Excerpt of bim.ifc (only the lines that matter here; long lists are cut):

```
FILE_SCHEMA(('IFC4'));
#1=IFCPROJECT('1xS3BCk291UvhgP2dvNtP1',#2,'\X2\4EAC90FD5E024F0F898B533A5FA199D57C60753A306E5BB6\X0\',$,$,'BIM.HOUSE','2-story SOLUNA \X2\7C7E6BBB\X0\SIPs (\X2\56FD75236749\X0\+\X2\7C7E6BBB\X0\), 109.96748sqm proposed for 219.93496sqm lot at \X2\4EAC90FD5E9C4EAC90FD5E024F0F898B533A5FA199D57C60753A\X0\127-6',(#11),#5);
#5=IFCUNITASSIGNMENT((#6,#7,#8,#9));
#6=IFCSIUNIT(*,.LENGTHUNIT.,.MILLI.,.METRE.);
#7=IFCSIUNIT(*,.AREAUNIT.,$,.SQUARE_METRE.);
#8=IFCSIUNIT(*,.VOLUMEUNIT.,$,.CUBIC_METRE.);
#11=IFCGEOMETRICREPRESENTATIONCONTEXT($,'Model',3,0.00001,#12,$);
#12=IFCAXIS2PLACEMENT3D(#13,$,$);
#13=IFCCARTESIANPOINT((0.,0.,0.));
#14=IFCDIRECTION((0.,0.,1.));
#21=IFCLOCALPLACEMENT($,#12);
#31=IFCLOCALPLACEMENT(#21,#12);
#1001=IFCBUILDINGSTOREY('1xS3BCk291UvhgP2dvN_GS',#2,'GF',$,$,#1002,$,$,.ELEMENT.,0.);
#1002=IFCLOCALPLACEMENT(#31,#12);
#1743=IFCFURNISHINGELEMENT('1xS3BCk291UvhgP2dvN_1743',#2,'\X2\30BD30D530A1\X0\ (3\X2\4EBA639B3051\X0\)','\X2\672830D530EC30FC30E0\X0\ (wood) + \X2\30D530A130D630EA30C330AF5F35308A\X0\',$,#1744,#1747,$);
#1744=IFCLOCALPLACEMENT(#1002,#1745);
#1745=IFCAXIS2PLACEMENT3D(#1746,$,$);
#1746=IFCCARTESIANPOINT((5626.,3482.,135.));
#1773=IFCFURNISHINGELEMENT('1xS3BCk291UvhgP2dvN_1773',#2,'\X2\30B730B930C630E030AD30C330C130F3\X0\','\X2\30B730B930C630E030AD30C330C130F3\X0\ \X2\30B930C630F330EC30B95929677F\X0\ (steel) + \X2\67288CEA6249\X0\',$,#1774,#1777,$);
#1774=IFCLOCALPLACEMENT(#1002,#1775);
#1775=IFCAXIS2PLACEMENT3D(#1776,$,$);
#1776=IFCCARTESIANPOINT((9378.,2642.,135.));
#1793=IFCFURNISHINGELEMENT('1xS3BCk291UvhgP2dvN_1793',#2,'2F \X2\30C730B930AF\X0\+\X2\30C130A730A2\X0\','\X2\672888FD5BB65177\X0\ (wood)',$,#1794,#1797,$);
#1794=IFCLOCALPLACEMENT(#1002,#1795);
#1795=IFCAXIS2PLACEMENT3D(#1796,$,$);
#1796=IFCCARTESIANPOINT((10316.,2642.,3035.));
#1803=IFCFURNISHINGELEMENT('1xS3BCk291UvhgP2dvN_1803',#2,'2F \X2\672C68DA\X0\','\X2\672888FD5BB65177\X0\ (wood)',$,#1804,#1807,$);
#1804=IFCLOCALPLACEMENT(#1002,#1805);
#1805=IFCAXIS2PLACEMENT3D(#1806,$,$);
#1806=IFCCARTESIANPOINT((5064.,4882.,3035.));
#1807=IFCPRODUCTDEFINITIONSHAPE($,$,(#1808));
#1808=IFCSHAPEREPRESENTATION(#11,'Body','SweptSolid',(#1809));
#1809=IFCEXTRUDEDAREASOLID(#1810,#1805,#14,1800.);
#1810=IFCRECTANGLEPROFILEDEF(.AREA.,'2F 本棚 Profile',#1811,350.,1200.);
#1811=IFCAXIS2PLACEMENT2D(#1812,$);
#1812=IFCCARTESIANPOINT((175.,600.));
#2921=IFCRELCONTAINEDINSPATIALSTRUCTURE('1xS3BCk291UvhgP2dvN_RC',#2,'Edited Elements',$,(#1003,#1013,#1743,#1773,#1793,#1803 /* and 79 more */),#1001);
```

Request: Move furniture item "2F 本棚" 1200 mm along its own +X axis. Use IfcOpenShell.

```python
import ifcopenshell
import ifcopenshell.api.geometry
import ifcopenshell.util.placement
import ifcopenshell.util.unit

model = ifcopenshell.open("bim.ifc")
unit_scale = ifcopenshell.util.unit.calculate_unit_scale(model)

item = model.by_id(1803)
matrix = ifcopenshell.util.placement.get_local_placement(item.ObjectPlacement)
matrix[:3, 3] += matrix[:3, 0] * 1.2 / unit_scale
ifcopenshell.api.geometry.edit_object_placement(model, product=item, matrix=matrix, is_si=False)

print(ifcopenshell.util.placement.get_local_placement(item.ObjectPlacement).round(3) + 0.0)

model.write("bim_updated.ifc")
```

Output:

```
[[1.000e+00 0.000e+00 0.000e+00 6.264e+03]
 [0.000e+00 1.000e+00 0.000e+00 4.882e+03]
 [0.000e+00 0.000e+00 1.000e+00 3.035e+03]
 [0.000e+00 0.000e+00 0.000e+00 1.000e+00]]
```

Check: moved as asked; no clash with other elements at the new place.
